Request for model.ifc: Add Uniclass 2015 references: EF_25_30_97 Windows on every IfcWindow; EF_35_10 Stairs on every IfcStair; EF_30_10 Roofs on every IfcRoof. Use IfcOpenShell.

First a look at what the model holds.

```python
import ifcopenshell

model = ifcopenshell.open("model.ifc")
print(model.schema)
print("classifications:", [c.Name for c in model.by_type("IfcClassification")])
for ifc_class in ("IfcDoor", "IfcRoof", "IfcStair", "IfcWall", "IfcWindow"):
    print(ifc_class, len(model.by_type(ifc_class)))
```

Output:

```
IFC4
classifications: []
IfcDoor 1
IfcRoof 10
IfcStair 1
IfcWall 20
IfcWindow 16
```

```python
import ifcopenshell
import ifcopenshell.api.classification

model = ifcopenshell.open("model.ifc")

system = ifcopenshell.api.classification.add_classification(model, classification="Uniclass 2015")

codes = {
    "IfcWindow": ("EF_25_30_97", "Windows"),
    "IfcStair": ("EF_35_10", "Stairs"),
    "IfcRoof": ("EF_30_10", "Roofs"),
}
for ifc_class, (code, name) in codes.items():
    products = model.by_type(ifc_class)
    ifcopenshell.api.classification.add_reference(
        model, products=products, classification=system, identification=code, name=name
    )
    print(code, len(products))

model.write("model_edited.ifc")
```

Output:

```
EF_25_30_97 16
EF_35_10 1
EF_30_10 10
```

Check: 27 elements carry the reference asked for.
